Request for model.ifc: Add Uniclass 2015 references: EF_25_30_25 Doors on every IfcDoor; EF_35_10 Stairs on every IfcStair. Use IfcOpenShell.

First a look at what the model holds.

```python
import ifcopenshell

model = ifcopenshell.open("model.ifc")
print(model.schema)
print("classifications:", [c.Name for c in model.by_type("IfcClassification")])
for ifc_class in ("IfcDoor", "IfcRoof", "IfcStair", "IfcWall", "IfcWindow"):
    print(ifc_class, len(model.by_type(ifc_class)))
```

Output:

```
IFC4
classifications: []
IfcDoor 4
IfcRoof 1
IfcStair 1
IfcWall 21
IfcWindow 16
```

```python
import ifcopenshell
import ifcopenshell.api.classification

model = ifcopenshell.open("model.ifc")

system = ifcopenshell.api.classification.add_classification(model, classification="Uniclass 2015")

codes = {
    "IfcDoor": ("EF_25_30_25", "Doors"),
    "IfcStair": ("EF_35_10", "Stairs"),
}
for ifc_class, (code, name) in codes.items():
    products = model.by_type(ifc_class)
    ifcopenshell.api.classification.add_reference(
        model, products=products, classification=system, identification=code, name=name
    )
    print(code, len(products))

model.write("model_updated.ifc")
```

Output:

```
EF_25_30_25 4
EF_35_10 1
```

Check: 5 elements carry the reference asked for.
